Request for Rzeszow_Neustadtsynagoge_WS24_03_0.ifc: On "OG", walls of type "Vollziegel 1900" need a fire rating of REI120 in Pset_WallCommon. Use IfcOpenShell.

First a look at what the model holds.

```python
import ifcopenshell
import ifcopenshell.util.element

model = ifcopenshell.open("Rzeszow_Neustadtsynagoge_WS24_03_0.ifc")
print(model.schema)
storey = next(s for s in model.by_type("IfcBuildingStorey") if s.Name == "OG")
walls = [e for e in ifcopenshell.util.element.get_decomposition(storey) if e.is_a("IfcWall")]
seen = {}
for e in walls:
    element_type = ifcopenshell.util.element.get_type(e)
    key = (element_type.Name if element_type != e and element_type else None, ifcopenshell.util.element.get_pset(e, "Pset_WallCommon", "FireRating"))
    seen[key] = seen.get(key, 0) + 1
for (name, value), count in sorted(seen.items(), key=str):
    print(count, "x", name, "|", value)
```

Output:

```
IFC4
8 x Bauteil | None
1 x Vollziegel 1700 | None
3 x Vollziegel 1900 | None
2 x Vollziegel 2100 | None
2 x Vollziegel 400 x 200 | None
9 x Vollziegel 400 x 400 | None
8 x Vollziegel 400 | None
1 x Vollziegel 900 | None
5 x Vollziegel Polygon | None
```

```python
import ifcopenshell
import ifcopenshell.api.pset
import ifcopenshell.util.element

model = ifcopenshell.open("Rzeszow_Neustadtsynagoge_WS24_03_0.ifc")

storey = next(s for s in model.by_type("IfcBuildingStorey") if s.Name == "OG")
walls = [e for e in ifcopenshell.util.element.get_decomposition(storey) if e.is_a("IfcWall")]

count = 0
for e in walls:
    element_type = ifcopenshell.util.element.get_type(e)
    if element_type in (None, e) or element_type.Name != "Vollziegel 1900":
        continue
    # add_pset returns the element's existing set when there is one.
    pset = ifcopenshell.api.pset.add_pset(model, product=e, name="Pset_WallCommon")
    ifcopenshell.api.pset.edit_pset(model, pset=pset, properties={"FireRating": "REI120"})
    count += 1

print(count, "walls updated")

model.write("Rzeszow_Neustadtsynagoge_WS24_03_0_updated.ifc")
```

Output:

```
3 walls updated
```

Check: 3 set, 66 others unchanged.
